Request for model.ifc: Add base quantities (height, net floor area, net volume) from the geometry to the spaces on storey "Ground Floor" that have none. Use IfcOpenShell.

First a look at what the model holds.

```python
import ifcopenshell
import ifcopenshell.util.element
import ifcopenshell.util.unit

model = ifcopenshell.open("model.ifc")
print(model.schema)
for unit_type in ("LENGTHUNIT", "AREAUNIT", "VOLUMEUNIT"):
    print(unit_type, ifcopenshell.util.unit.calculate_unit_scale(model, unit_type))
storey = next(s for s in model.by_type("IfcBuildingStorey") if s.Name == "Ground Floor")
spaces = [e for e in ifcopenshell.util.element.get_decomposition(storey) if e.is_a("IfcSpace")]
for e in sorted(spaces, key=lambda e: e.id()):
    print(e.id(), e.is_a(), e.Name, list(ifcopenshell.util.element.get_psets(e, qtos_only=True)), sep=" | ")
```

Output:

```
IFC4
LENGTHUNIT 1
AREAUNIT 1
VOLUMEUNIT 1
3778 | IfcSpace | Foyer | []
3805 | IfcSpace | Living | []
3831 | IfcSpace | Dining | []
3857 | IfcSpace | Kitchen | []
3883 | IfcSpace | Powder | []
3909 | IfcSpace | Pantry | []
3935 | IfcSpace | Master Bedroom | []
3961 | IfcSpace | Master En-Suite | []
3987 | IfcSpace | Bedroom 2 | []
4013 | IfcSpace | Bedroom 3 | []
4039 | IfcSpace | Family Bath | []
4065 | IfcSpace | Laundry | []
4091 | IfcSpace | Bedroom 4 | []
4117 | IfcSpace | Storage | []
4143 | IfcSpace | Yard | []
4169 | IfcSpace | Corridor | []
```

```python
import ifcopenshell
import ifcopenshell.api.pset
import ifcopenshell.geom
import ifcopenshell.util.element
import ifcopenshell.util.shape
import ifcopenshell.util.unit

model = ifcopenshell.open("model.ifc")
unit_scale = ifcopenshell.util.unit.calculate_unit_scale(model)
area_scale = ifcopenshell.util.unit.calculate_unit_scale(model, "AREAUNIT")
volume_scale = ifcopenshell.util.unit.calculate_unit_scale(model, "VOLUMEUNIT")
settings = ifcopenshell.geom.settings()

storey = next(s for s in model.by_type("IfcBuildingStorey") if s.Name == "Ground Floor")
spaces = [e for e in ifcopenshell.util.element.get_decomposition(storey) if e.is_a("IfcSpace")]

for e in sorted(spaces, key=lambda e: e.id()):
    if ifcopenshell.util.element.get_psets(e, qtos_only=True, should_inherit=False):
        continue
    # Geometry comes back in metres, in the element's own axes.
    shape = ifcopenshell.geom.create_shape(settings, e)
    values = {
        "Height": ifcopenshell.util.shape.get_z(shape.geometry) / unit_scale,
        "NetFloorArea": ifcopenshell.util.shape.get_footprint_area(shape.geometry) / area_scale,
        "NetVolume": ifcopenshell.util.shape.get_volume(shape.geometry) / volume_scale,
    }
    qto = ifcopenshell.api.pset.add_qto(model, product=e, name="Qto_SpaceBaseQuantities")
    ifcopenshell.api.pset.edit_qto(model, qto=qto, properties=values)
    print(e.id(), {k: round(v, 3) for k, v in values.items()})

model.write("model-out.ifc")
```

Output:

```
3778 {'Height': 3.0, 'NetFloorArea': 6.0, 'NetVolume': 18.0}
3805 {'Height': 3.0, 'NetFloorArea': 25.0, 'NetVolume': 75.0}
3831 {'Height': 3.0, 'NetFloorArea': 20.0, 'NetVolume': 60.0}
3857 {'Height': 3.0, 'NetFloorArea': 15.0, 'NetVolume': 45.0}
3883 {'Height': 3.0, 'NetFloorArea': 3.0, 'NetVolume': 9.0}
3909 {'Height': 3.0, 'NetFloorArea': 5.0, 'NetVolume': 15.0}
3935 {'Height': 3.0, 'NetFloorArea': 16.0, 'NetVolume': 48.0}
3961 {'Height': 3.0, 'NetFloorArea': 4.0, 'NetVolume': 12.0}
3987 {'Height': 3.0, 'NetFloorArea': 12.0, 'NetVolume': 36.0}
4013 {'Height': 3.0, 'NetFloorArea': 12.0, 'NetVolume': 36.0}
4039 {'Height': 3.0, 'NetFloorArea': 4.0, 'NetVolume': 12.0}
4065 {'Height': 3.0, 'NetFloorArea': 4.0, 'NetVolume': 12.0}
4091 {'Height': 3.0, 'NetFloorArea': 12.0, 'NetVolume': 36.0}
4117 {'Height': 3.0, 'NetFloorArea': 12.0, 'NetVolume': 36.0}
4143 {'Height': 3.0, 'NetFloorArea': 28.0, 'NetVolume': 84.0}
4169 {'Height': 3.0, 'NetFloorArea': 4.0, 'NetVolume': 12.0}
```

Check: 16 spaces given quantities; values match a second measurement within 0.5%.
